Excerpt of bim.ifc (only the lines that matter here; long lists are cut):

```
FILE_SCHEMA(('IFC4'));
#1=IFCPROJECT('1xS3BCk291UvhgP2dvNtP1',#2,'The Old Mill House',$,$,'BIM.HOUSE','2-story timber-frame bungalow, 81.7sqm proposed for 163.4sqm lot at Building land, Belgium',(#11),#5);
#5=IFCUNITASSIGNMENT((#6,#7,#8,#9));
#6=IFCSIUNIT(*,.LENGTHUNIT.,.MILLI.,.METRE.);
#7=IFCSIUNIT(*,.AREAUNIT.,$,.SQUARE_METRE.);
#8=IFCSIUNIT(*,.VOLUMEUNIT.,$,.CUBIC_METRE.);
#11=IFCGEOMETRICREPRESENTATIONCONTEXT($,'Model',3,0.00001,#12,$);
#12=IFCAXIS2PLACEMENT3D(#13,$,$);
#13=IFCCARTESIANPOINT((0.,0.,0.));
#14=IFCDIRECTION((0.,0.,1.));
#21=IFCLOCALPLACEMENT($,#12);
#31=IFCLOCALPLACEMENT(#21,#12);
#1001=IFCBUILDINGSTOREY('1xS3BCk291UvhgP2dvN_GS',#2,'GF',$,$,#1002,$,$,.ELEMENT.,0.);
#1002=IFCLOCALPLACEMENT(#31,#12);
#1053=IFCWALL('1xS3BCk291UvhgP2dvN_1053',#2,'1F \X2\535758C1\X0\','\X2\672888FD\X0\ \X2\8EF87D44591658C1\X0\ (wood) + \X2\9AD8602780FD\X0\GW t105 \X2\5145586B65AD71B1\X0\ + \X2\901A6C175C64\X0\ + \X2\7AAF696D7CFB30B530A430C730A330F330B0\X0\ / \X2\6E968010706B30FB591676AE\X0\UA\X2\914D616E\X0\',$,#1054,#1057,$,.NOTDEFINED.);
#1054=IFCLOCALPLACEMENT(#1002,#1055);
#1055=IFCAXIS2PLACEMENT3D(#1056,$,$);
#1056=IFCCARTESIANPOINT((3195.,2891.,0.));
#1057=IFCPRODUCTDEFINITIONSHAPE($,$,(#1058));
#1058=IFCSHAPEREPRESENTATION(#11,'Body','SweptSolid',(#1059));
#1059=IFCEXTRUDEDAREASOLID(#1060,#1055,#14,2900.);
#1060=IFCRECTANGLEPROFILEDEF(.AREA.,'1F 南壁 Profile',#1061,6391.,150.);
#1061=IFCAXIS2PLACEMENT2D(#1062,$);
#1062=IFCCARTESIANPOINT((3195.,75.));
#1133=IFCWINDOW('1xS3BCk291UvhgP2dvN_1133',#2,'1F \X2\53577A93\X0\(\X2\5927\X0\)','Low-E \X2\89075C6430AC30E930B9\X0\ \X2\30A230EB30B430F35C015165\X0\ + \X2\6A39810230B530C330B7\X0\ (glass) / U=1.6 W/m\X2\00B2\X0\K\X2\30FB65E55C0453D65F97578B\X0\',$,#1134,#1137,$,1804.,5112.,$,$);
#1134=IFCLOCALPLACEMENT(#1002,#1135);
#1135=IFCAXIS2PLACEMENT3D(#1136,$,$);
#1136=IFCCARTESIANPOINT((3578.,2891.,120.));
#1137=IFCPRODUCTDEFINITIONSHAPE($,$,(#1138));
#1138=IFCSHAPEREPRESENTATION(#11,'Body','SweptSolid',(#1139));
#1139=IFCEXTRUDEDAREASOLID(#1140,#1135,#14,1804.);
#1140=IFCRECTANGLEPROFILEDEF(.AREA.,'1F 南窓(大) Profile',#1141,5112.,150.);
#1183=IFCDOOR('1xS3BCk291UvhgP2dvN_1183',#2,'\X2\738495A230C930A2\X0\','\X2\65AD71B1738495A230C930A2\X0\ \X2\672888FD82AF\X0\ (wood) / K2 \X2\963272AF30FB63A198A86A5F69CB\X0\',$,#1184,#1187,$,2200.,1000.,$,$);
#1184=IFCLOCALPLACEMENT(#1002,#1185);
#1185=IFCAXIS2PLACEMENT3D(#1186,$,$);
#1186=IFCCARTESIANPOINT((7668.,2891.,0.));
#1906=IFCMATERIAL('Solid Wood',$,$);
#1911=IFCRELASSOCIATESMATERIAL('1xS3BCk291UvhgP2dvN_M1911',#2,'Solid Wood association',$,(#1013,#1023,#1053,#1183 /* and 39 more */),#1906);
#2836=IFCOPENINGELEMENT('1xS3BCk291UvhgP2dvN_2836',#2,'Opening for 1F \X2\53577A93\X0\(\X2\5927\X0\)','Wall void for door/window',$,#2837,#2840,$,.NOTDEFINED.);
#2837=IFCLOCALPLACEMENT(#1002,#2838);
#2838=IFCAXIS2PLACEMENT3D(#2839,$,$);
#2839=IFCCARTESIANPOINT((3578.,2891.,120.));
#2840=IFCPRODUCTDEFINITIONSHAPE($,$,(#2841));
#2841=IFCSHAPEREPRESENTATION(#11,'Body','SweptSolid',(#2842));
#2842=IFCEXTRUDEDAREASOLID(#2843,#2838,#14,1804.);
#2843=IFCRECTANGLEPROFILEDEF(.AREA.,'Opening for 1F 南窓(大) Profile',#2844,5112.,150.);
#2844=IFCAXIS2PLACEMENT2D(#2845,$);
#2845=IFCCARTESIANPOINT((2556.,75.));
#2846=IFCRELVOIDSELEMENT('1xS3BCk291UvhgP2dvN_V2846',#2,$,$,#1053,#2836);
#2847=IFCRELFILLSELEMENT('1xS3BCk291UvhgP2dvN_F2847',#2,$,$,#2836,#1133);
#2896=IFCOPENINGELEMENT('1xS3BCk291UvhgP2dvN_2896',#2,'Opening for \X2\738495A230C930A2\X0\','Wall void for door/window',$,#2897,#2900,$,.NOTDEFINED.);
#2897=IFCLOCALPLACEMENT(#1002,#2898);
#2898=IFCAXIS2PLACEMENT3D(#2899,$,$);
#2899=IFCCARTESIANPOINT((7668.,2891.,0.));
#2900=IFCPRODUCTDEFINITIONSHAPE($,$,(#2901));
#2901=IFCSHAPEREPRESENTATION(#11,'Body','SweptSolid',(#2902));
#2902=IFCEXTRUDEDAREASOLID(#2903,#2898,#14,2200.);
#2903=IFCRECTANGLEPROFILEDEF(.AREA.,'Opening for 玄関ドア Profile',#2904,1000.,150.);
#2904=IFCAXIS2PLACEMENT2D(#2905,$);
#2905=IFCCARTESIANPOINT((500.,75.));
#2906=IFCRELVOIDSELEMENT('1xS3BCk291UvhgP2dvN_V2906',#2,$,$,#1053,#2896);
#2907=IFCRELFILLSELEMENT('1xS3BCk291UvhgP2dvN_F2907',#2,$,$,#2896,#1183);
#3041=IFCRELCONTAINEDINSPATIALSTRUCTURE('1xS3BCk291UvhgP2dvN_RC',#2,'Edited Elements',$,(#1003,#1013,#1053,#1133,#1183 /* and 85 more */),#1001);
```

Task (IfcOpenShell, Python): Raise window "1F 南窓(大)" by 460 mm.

```python
import numpy as np
import ifcopenshell
import ifcopenshell.api.geometry
import ifcopenshell.util.placement
import ifcopenshell.util.unit

model = ifcopenshell.open("bim.ifc")
unit_scale = ifcopenshell.util.unit.calculate_unit_scale(model)

window = model.by_guid("1xS3BCk291UvhgP2dvN_1133")
opening = window.FillsVoids[0].RelatingOpeningElement
dz = 0.46 / unit_scale

shift = np.array([0.0, 0.0, dz])
# The window is not placed relative to its opening, so move both.
for product in (opening, window):
    matrix = ifcopenshell.util.placement.get_local_placement(product.ObjectPlacement)
    matrix[:3, 3] += shift
    ifcopenshell.api.geometry.edit_object_placement(model, product=product, matrix=matrix, is_si=False)

print(f"moved by {dz * unit_scale:+.3f} m")

model.write("bim_edited.ifc")
```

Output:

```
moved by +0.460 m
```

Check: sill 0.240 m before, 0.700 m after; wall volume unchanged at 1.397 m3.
